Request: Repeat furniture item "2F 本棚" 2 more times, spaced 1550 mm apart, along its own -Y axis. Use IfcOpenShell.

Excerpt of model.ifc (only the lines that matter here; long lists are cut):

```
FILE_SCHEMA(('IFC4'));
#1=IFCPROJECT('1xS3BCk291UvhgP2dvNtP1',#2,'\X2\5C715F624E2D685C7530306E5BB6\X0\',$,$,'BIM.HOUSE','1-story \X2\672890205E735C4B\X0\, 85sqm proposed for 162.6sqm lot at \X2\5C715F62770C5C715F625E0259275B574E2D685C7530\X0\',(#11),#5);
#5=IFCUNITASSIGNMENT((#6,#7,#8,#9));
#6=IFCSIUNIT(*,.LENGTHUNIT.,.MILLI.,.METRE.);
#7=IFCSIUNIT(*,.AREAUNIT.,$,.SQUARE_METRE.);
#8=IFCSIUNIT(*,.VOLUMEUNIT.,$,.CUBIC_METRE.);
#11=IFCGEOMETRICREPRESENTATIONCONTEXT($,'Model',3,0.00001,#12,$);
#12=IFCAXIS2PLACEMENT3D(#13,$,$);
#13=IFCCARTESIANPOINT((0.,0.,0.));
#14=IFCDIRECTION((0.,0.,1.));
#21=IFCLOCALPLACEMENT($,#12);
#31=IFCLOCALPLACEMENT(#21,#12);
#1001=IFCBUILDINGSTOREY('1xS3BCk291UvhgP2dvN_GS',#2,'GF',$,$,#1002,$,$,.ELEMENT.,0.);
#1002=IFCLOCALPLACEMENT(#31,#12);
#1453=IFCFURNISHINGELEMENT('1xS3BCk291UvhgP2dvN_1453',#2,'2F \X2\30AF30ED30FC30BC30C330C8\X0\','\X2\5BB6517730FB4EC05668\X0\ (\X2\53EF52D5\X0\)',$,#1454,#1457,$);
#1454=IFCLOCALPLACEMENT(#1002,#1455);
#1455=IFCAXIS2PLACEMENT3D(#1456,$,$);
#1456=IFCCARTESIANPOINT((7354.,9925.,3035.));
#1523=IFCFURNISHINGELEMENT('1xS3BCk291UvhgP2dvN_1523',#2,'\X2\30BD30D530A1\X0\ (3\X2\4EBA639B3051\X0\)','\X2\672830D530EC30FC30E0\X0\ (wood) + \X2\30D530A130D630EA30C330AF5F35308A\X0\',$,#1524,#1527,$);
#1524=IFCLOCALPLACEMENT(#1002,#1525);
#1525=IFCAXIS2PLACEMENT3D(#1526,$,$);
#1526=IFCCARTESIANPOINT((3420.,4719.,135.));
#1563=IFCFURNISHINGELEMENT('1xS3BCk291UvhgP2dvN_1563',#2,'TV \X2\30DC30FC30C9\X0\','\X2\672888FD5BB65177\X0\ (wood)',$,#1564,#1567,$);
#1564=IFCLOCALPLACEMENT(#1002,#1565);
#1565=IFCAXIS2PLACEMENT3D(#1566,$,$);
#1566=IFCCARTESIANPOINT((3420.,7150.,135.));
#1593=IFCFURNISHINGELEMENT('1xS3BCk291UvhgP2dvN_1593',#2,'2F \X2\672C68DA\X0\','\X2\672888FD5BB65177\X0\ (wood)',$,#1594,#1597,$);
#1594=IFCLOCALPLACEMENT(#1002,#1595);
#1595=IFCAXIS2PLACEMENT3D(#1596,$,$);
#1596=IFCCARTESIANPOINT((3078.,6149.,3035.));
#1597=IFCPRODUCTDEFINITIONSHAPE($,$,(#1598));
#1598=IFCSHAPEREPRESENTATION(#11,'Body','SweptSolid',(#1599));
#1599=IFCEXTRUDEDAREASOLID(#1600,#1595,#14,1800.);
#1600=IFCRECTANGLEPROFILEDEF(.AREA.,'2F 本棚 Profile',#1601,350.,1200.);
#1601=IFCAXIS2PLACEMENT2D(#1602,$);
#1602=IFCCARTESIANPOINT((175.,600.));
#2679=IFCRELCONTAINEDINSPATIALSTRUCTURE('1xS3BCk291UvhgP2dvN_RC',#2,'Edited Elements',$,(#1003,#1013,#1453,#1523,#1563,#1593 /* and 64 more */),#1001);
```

```python
import ifcopenshell
import ifcopenshell.api.geometry
import ifcopenshell.api.root
import ifcopenshell.util.element
import ifcopenshell.util.placement
import ifcopenshell.util.unit

model = ifcopenshell.open("model.ifc")
unit_scale = ifcopenshell.util.unit.calculate_unit_scale(model)


def reuse_history(source, copy):
    """copy_class also copies each property set's owner history, people and application; keep the originals."""
    for rel in copy.IsDefinedBy:
        if rel.is_a("IfcRelDefinesByProperties") and (history := rel.RelatingPropertyDefinition.OwnerHistory):
            rel.RelatingPropertyDefinition.OwnerHistory = source.OwnerHistory
            ifcopenshell.util.element.remove_deep2(model, history)


source = model.by_id(1593)
base = ifcopenshell.util.placement.get_local_placement(source.ObjectPlacement)
step = -base[:3, 1] * 1.55 / unit_scale

for i in range(1, 3):
    copy = ifcopenshell.api.root.copy_class(model, product=source)
    copy.Representation = ifcopenshell.util.element.copy_deep(
        model, source.Representation, exclude=["IfcGeometricRepresentationContext", "IfcRepresentationMap"]
    )
    reuse_history(source, copy)
    matrix = base.copy()
    matrix[:3, 3] += i * step
    print("added at", matrix[:3, 3].round(3) + 0.0)
    ifcopenshell.api.geometry.edit_object_placement(model, product=copy, matrix=matrix, is_si=False)

model.write("model_edited.ifc")
```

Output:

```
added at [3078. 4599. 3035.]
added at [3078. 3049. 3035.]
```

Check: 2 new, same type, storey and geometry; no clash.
